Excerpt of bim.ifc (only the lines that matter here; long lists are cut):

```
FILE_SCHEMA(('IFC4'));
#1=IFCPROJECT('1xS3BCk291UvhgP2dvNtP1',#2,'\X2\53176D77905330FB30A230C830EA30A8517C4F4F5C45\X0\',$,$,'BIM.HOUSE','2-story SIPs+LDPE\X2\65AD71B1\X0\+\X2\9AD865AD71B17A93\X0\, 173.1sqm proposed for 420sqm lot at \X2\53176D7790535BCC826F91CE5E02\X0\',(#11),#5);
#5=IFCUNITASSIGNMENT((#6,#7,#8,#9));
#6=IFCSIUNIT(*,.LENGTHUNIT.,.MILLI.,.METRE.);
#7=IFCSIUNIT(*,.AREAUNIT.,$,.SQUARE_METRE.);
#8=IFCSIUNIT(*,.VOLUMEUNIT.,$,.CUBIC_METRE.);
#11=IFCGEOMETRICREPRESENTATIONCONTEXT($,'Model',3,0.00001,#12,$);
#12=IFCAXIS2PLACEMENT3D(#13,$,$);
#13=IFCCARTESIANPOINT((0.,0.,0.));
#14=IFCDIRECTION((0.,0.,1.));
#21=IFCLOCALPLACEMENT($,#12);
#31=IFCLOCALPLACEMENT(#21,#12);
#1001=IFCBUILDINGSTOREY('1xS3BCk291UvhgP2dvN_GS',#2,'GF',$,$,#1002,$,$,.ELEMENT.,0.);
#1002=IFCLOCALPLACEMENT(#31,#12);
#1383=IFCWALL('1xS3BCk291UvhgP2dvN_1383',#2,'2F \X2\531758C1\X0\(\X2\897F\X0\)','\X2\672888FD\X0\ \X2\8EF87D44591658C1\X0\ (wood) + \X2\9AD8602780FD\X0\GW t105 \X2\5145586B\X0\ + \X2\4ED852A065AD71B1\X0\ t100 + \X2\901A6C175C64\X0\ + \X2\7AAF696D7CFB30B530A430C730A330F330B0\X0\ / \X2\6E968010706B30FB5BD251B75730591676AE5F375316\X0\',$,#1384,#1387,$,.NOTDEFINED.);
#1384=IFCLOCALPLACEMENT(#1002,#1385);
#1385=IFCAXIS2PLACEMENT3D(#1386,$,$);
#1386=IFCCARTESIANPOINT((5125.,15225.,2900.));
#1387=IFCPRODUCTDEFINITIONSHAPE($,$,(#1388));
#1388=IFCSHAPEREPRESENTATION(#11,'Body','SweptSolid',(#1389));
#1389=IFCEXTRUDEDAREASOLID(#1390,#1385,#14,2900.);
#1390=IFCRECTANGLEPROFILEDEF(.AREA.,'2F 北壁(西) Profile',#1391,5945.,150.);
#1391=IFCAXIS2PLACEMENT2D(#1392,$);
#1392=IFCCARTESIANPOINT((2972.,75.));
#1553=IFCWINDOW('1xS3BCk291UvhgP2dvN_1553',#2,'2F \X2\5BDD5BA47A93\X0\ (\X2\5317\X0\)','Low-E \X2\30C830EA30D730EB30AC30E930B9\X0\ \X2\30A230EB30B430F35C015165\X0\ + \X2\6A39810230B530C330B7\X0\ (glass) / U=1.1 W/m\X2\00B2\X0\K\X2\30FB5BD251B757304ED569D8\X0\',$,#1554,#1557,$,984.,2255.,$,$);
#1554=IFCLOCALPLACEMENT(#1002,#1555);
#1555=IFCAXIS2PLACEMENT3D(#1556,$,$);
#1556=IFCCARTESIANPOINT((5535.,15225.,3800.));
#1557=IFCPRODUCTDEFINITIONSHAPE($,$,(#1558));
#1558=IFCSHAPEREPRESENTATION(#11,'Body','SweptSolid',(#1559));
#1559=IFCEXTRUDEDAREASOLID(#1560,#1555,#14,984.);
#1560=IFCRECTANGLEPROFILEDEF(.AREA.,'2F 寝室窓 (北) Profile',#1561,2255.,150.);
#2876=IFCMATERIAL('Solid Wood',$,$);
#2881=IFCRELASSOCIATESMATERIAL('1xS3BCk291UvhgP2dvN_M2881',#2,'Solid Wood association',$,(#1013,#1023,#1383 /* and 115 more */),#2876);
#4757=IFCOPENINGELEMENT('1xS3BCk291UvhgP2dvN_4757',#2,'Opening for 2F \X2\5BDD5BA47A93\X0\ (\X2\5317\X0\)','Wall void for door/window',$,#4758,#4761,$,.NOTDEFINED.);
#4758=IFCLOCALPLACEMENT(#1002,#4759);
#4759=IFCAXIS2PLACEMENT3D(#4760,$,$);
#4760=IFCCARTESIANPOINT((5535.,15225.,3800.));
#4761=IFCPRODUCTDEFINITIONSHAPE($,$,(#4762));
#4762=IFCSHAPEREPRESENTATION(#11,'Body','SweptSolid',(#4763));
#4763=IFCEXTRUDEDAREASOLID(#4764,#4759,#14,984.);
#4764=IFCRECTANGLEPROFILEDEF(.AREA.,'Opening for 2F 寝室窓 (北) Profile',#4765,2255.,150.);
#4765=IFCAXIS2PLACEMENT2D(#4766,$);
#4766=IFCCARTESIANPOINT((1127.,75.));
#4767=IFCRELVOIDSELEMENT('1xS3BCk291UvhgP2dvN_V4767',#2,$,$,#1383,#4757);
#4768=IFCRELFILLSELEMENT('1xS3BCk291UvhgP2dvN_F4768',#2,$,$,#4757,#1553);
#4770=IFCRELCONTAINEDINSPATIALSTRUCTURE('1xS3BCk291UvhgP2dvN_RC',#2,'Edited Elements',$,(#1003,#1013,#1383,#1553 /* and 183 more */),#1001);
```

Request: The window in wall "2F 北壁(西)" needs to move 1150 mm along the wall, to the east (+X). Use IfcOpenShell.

```python
import ifcopenshell
import ifcopenshell.api.geometry
import ifcopenshell.util.placement

model = ifcopenshell.open("bim.ifc")

window = model.by_id(1553)
opening = window.FillsVoids[0].RelatingOpeningElement
wall = opening.VoidsElements[0].RelatingBuildingElement

wall_matrix = ifcopenshell.util.placement.get_local_placement(wall.ObjectPlacement)
shift = wall_matrix[:3, 0] * 1150.0
before = ifcopenshell.util.placement.get_local_placement(window.ObjectPlacement)[:3, 3].copy()

# The window is not placed relative to its opening, so move both.
for product in (opening, window):
    matrix = ifcopenshell.util.placement.get_local_placement(product.ObjectPlacement)
    matrix[:3, 3] += shift
    ifcopenshell.api.geometry.edit_object_placement(model, product=product, matrix=matrix, is_si=False)

after = ifcopenshell.util.placement.get_local_placement(window.ObjectPlacement)[:3, 3]
print("window moved by", (after - before).round(3) + 0.0)

model.write("bim_v2.ifc")
```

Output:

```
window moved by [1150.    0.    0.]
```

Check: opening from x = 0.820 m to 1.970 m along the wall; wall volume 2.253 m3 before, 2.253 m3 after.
